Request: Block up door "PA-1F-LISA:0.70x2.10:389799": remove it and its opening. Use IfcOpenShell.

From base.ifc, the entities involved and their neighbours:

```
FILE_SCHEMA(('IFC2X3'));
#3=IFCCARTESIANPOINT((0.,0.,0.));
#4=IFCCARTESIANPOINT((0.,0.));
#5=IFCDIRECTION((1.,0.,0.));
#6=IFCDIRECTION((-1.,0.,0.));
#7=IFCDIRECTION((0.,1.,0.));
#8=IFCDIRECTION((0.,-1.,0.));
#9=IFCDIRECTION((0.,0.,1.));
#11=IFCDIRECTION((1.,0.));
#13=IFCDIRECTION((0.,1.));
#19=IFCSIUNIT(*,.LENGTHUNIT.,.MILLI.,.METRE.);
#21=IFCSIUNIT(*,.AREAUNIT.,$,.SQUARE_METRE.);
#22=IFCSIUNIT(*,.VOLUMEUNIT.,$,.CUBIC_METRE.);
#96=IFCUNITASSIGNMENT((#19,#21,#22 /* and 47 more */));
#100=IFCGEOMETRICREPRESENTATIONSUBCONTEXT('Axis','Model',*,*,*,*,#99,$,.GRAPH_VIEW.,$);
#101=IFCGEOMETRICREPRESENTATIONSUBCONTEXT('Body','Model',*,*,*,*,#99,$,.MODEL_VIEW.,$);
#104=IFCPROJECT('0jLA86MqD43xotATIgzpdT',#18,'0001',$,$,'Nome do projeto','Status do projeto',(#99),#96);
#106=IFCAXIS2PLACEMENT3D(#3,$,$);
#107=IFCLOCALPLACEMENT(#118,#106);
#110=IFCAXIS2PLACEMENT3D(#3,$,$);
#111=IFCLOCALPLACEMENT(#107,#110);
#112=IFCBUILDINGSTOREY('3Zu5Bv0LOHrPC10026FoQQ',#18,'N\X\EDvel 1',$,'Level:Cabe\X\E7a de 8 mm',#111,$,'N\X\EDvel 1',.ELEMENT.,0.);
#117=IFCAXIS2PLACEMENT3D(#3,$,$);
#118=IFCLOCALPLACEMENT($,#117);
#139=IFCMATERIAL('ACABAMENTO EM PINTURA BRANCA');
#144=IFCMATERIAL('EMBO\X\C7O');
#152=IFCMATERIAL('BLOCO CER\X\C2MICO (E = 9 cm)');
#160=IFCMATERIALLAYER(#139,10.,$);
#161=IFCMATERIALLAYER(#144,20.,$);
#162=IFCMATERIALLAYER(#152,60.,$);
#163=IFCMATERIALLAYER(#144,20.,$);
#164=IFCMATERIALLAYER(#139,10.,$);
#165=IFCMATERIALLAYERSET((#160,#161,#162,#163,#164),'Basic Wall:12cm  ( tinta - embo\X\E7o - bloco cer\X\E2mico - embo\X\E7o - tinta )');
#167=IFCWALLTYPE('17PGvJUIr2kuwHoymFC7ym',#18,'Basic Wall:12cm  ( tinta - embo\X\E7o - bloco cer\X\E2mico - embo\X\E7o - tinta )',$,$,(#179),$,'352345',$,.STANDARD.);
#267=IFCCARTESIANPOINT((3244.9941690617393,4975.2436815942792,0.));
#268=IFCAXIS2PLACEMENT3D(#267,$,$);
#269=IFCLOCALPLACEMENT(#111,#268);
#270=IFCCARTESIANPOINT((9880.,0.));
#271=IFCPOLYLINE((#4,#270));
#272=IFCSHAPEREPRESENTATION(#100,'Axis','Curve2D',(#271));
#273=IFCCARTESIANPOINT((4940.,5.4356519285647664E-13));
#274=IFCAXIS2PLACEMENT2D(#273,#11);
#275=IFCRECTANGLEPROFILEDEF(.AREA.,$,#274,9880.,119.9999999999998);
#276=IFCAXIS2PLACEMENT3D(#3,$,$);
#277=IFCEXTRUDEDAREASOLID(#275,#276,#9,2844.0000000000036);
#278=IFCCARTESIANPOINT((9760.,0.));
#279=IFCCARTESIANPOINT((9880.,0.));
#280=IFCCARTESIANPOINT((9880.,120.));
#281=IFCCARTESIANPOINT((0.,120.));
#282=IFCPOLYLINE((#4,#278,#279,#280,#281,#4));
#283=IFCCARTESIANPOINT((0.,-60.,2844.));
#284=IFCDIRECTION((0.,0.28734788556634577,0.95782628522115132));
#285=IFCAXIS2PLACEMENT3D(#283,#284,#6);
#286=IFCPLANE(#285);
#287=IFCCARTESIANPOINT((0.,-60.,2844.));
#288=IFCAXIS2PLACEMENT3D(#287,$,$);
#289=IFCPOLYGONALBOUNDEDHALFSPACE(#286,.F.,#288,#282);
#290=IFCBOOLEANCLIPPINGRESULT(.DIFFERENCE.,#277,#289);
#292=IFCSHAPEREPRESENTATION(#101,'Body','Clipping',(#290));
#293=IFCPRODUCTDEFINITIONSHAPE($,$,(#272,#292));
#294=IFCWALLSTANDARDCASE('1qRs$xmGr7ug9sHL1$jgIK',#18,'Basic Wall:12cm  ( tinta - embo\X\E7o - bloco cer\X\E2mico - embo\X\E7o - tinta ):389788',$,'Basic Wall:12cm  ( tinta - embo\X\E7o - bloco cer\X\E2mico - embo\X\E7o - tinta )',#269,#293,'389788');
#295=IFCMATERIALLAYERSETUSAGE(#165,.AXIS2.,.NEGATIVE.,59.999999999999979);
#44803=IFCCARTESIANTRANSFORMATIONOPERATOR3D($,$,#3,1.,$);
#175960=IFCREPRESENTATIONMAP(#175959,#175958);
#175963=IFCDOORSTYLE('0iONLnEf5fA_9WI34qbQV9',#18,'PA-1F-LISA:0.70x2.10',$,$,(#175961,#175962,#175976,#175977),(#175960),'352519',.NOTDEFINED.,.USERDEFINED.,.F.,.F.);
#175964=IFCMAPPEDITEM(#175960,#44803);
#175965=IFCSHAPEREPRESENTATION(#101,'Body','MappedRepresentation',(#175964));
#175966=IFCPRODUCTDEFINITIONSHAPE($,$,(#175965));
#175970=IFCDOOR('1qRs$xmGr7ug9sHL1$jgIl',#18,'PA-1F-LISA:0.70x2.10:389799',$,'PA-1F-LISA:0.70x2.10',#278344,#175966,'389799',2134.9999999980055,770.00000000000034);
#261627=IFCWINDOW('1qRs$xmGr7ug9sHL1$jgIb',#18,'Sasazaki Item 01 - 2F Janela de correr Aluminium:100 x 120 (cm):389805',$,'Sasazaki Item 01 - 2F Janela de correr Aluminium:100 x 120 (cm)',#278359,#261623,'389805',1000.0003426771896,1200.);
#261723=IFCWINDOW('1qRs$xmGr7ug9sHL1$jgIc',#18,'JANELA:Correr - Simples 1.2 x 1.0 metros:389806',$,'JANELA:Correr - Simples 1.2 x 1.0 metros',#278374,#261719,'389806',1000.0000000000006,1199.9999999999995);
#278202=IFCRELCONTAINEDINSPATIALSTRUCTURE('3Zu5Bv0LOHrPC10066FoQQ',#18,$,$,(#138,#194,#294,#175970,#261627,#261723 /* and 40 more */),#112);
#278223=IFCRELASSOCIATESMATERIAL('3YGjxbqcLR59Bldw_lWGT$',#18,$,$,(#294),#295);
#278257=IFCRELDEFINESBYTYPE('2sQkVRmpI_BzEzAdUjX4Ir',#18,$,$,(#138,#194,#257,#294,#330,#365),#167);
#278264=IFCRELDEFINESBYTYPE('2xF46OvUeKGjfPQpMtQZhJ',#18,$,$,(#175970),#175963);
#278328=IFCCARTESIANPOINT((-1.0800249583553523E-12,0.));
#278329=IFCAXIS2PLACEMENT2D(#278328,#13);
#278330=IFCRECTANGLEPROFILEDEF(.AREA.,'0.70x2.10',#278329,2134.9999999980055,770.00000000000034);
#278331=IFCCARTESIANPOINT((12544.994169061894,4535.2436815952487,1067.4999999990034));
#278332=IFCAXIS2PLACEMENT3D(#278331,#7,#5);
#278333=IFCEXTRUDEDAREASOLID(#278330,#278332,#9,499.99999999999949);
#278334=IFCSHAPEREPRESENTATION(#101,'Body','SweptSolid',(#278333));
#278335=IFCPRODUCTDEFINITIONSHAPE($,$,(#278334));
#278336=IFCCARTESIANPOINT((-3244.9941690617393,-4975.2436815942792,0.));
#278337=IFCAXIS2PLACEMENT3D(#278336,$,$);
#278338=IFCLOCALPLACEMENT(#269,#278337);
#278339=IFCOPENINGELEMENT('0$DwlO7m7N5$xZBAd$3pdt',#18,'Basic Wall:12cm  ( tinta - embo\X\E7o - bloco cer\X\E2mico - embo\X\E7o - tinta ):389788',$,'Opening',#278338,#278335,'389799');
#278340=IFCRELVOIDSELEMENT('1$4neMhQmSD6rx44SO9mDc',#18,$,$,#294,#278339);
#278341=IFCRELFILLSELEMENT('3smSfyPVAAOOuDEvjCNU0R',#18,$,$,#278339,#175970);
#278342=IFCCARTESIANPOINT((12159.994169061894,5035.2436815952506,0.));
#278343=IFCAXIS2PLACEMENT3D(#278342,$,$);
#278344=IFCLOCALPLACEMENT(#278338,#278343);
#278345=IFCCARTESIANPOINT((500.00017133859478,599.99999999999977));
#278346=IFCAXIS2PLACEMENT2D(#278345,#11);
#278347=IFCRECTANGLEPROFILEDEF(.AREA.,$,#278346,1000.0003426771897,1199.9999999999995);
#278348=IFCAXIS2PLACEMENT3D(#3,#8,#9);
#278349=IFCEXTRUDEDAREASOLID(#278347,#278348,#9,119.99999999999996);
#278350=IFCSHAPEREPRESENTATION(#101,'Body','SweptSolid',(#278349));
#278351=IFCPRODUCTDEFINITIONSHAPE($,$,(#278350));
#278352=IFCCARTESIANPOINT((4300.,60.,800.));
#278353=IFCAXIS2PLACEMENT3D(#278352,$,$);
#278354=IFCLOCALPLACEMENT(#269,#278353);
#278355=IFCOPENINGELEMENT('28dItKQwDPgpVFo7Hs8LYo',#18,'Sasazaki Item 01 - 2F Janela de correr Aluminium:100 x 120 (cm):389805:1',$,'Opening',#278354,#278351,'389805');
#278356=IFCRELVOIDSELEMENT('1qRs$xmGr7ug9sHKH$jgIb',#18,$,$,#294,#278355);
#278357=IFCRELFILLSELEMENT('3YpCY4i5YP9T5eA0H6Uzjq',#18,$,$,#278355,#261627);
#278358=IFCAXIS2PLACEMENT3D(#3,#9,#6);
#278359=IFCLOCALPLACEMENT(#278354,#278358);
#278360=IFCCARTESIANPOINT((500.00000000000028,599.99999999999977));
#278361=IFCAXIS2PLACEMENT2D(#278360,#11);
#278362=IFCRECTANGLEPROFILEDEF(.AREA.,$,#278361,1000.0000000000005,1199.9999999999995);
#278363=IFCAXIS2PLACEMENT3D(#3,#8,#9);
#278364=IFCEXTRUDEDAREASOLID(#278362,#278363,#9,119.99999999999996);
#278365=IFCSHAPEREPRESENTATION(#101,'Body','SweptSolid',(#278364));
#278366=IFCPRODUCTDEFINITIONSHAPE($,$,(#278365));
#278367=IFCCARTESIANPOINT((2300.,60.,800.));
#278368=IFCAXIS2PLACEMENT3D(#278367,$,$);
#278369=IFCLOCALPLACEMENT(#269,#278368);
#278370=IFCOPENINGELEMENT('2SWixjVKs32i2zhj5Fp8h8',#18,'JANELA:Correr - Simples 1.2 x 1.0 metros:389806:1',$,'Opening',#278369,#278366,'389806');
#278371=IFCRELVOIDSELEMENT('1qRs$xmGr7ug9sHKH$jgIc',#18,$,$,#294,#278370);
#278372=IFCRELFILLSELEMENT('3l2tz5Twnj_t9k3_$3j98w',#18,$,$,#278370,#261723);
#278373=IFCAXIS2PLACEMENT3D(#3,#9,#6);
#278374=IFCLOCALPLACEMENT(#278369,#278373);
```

```python
import ifcopenshell
import ifcopenshell.api.feature
import ifcopenshell.api.root
import ifcopenshell.geom
import ifcopenshell.util.shape

model = ifcopenshell.open("base.ifc")
settings = ifcopenshell.geom.settings()


def volume(element):
    """Net volume in cubic metres, openings subtracted."""
    shape = ifcopenshell.geom.create_shape(settings, element)
    return ifcopenshell.util.shape.get_volume(shape.geometry)


door = model.by_guid("1qRs$xmGr7ug9sHL1$jgIl")
opening = door.FillsVoids[0].RelatingOpeningElement
wall = opening.VoidsElements[0].RelatingBuildingElement
before = volume(wall)

ifcopenshell.api.root.remove_product(model, product=door)
ifcopenshell.api.feature.remove_feature(model, feature=opening)

after = volume(wall)

print(f"wall volume {before:.3f} -> {after:.3f} m3")

model.write("base_rev.ifc")
```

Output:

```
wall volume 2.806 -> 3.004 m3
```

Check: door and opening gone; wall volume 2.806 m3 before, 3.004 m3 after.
